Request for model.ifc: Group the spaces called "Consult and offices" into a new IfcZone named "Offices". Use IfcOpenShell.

First a look at what the model holds.

```python
import ifcopenshell

model = ifcopenshell.open("model.ifc")
print(model.schema)
seen = {}
for space in model.by_type("IfcSpace"):
    seen[space.Name] = seen.get(space.Name, 0) + 1
for name, count in sorted(seen.items(), key=str):
    print(count, "x", name)
print("zones:", [z.Name for z in model.by_type("IfcZone")][:20])
```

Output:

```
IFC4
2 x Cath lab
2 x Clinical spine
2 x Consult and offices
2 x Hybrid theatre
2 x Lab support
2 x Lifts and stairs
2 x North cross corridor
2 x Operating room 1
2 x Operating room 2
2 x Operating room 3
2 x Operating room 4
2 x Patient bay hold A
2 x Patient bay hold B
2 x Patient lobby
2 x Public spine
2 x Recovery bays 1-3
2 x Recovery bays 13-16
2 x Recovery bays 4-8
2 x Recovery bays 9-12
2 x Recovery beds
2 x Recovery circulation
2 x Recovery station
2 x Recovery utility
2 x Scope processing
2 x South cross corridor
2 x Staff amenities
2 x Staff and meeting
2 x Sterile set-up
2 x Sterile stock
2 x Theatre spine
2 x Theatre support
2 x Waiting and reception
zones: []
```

```python
import ifcopenshell
import ifcopenshell.api.group
import ifcopenshell.api.root

model = ifcopenshell.open("model.ifc")

names = {"Consult and offices"}
spaces = [s for s in model.by_type("IfcSpace") if s.Name in names]

zone = ifcopenshell.api.root.create_entity(model, ifc_class="IfcZone", name="Offices")
ifcopenshell.api.group.assign_group(model, products=spaces, group=zone)
print(len(spaces), "spaces in", zone.Name)

model.write("model_updated.ifc")
```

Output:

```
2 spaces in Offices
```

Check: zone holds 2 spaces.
